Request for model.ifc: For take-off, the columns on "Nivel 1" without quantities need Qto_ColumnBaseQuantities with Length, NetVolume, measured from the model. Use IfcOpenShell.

First a look at what the model holds.

```python
import ifcopenshell
import ifcopenshell.util.element
import ifcopenshell.util.unit

model = ifcopenshell.open("model.ifc")
print(model.schema)
for unit_type in ("LENGTHUNIT", "AREAUNIT", "VOLUMEUNIT"):
    print(unit_type, ifcopenshell.util.unit.calculate_unit_scale(model, unit_type))
storey = next(s for s in model.by_type("IfcBuildingStorey") if s.Name == "Nivel 1")
columns = [e for e in ifcopenshell.util.element.get_decomposition(storey) if e.is_a("IfcColumn")]
for e in sorted(columns, key=lambda e: e.id()):
    print(e.id(), e.is_a(), e.Name, list(ifcopenshell.util.element.get_psets(e, qtos_only=True)), sep=" | ")
```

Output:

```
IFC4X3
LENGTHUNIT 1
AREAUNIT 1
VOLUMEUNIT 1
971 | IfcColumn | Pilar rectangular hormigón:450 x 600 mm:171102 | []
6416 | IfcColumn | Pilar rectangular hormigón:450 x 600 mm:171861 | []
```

```python
import ifcopenshell
import ifcopenshell.api.pset
import ifcopenshell.geom
import ifcopenshell.util.element
import ifcopenshell.util.shape
import ifcopenshell.util.unit

model = ifcopenshell.open("model.ifc")
unit_scale = ifcopenshell.util.unit.calculate_unit_scale(model)
volume_scale = ifcopenshell.util.unit.calculate_unit_scale(model, "VOLUMEUNIT")
settings = ifcopenshell.geom.settings()

storey = next(s for s in model.by_type("IfcBuildingStorey") if s.Name == "Nivel 1")
columns = [e for e in ifcopenshell.util.element.get_decomposition(storey) if e.is_a("IfcColumn")]

for e in sorted(columns, key=lambda e: e.id()):
    if ifcopenshell.util.element.get_psets(e, qtos_only=True, should_inherit=False):
        continue
    # Geometry comes back in metres, in the element's own axes.
    shape = ifcopenshell.geom.create_shape(settings, e)
    values = {
        "Length": ifcopenshell.util.shape.get_z(shape.geometry) / unit_scale,
        "NetVolume": ifcopenshell.util.shape.get_volume(shape.geometry) / volume_scale,
    }
    qto = ifcopenshell.api.pset.add_qto(model, product=e, name="Qto_ColumnBaseQuantities")
    ifcopenshell.api.pset.edit_qto(model, qto=qto, properties=values)
    print(e.id(), {k: round(v, 3) for k, v in values.items()})

model.write("model-out.ifc")
```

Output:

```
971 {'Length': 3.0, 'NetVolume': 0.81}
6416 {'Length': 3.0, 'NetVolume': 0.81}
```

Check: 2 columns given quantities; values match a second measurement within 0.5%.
